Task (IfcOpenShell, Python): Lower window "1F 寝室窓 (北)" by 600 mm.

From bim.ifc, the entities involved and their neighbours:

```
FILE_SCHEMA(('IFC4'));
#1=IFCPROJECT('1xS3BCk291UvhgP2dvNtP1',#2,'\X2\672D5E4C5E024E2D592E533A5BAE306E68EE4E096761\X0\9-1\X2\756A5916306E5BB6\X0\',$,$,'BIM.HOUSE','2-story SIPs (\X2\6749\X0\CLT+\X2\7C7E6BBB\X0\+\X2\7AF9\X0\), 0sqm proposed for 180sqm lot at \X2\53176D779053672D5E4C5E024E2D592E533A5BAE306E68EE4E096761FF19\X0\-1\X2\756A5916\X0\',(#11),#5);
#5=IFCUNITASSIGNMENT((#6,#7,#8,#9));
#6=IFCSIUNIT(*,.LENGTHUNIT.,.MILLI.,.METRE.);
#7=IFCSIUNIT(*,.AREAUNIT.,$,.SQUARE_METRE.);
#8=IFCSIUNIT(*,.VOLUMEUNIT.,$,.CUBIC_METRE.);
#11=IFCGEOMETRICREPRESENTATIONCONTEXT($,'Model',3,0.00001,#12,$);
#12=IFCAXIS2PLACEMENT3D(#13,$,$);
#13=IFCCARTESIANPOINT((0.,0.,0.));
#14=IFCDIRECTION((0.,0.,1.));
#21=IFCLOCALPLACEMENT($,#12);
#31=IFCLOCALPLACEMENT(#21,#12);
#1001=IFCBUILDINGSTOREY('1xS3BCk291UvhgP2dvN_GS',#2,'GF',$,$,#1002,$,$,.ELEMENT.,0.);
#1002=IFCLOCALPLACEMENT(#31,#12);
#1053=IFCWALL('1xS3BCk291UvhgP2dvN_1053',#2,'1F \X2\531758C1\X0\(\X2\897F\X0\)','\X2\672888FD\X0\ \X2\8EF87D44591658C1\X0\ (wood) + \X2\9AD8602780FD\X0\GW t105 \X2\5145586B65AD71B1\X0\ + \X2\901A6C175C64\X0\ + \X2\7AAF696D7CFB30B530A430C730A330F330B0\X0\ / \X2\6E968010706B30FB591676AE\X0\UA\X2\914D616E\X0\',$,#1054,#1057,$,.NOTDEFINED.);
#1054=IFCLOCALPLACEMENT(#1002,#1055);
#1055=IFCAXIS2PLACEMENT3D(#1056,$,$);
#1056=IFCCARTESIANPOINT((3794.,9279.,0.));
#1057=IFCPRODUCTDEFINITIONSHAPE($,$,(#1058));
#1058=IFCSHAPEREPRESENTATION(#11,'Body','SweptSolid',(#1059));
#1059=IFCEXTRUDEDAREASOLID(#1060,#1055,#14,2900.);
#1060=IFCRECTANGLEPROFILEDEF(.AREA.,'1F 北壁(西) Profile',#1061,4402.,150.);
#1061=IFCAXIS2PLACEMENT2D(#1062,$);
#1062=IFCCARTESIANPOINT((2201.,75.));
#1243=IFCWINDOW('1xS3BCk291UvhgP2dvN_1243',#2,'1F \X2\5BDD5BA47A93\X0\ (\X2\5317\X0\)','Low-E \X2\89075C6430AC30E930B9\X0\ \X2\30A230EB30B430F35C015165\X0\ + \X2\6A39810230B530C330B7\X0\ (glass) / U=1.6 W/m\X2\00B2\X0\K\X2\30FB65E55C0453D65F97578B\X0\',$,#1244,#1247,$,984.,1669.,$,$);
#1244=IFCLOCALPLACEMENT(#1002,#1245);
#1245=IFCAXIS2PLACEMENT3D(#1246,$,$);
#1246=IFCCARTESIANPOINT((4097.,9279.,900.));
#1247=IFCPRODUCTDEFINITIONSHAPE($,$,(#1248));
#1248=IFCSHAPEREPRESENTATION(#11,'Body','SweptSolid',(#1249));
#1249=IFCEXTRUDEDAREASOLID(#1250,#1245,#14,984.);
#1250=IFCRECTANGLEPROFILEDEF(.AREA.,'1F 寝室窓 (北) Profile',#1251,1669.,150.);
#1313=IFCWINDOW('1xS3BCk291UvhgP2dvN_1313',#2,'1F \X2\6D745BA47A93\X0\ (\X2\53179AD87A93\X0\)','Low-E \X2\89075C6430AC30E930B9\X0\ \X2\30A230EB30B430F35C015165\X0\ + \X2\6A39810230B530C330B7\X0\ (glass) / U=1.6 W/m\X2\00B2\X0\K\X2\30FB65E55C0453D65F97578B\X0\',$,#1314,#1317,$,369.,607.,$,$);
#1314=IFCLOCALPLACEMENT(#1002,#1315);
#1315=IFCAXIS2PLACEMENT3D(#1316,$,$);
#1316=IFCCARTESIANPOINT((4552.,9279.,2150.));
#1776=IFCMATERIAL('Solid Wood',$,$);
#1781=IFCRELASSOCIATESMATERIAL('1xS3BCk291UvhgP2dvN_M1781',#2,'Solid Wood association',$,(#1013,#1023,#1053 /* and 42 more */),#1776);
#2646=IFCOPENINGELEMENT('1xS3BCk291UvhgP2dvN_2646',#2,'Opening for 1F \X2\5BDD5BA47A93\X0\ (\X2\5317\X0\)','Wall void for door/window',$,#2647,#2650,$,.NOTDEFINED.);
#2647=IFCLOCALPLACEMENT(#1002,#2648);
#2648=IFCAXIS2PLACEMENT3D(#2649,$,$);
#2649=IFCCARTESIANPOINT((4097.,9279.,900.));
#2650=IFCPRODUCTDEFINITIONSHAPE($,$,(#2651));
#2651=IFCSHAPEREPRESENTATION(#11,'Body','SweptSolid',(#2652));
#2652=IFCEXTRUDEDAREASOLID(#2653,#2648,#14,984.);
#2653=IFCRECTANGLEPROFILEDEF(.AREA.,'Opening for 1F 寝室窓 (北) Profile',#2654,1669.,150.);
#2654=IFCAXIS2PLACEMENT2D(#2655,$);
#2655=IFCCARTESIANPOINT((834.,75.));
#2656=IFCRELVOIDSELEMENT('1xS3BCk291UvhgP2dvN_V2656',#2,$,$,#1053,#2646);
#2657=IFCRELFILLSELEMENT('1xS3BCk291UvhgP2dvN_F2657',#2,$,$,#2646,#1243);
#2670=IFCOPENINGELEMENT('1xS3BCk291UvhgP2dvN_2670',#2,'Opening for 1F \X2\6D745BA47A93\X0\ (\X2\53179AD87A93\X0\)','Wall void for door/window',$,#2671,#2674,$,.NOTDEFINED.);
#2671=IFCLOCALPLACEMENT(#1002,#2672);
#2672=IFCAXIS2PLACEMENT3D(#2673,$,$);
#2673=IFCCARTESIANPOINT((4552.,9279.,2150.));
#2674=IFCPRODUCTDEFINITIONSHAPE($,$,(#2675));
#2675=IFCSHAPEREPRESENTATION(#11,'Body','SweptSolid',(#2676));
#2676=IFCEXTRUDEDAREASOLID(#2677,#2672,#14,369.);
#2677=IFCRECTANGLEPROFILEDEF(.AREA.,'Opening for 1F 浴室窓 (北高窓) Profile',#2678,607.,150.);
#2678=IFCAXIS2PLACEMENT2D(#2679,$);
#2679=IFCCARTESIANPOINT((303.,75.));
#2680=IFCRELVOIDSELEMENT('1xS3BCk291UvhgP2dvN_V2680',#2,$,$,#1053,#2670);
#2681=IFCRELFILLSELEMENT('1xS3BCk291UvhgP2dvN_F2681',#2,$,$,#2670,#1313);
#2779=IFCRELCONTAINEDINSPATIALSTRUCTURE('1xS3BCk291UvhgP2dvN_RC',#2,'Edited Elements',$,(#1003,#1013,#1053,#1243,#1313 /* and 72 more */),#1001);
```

```python
import numpy as np
import ifcopenshell
import ifcopenshell.api.geometry
import ifcopenshell.util.placement
import ifcopenshell.util.unit

model = ifcopenshell.open("bim.ifc")
unit_scale = ifcopenshell.util.unit.calculate_unit_scale(model)

window = model.by_guid("1xS3BCk291UvhgP2dvN_1243")
opening = window.FillsVoids[0].RelatingOpeningElement
dz = -0.6 / unit_scale

shift = np.array([0.0, 0.0, dz])
# The window is not placed relative to its opening, so move both.
for product in (opening, window):
    matrix = ifcopenshell.util.placement.get_local_placement(product.ObjectPlacement)
    matrix[:3, 3] += shift
    ifcopenshell.api.geometry.edit_object_placement(model, product=product, matrix=matrix, is_si=False)

print(f"moved by {dz * unit_scale:+.3f} m")

model.write("bim_rev.ifc")
```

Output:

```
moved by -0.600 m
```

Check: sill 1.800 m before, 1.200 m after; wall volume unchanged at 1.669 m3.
